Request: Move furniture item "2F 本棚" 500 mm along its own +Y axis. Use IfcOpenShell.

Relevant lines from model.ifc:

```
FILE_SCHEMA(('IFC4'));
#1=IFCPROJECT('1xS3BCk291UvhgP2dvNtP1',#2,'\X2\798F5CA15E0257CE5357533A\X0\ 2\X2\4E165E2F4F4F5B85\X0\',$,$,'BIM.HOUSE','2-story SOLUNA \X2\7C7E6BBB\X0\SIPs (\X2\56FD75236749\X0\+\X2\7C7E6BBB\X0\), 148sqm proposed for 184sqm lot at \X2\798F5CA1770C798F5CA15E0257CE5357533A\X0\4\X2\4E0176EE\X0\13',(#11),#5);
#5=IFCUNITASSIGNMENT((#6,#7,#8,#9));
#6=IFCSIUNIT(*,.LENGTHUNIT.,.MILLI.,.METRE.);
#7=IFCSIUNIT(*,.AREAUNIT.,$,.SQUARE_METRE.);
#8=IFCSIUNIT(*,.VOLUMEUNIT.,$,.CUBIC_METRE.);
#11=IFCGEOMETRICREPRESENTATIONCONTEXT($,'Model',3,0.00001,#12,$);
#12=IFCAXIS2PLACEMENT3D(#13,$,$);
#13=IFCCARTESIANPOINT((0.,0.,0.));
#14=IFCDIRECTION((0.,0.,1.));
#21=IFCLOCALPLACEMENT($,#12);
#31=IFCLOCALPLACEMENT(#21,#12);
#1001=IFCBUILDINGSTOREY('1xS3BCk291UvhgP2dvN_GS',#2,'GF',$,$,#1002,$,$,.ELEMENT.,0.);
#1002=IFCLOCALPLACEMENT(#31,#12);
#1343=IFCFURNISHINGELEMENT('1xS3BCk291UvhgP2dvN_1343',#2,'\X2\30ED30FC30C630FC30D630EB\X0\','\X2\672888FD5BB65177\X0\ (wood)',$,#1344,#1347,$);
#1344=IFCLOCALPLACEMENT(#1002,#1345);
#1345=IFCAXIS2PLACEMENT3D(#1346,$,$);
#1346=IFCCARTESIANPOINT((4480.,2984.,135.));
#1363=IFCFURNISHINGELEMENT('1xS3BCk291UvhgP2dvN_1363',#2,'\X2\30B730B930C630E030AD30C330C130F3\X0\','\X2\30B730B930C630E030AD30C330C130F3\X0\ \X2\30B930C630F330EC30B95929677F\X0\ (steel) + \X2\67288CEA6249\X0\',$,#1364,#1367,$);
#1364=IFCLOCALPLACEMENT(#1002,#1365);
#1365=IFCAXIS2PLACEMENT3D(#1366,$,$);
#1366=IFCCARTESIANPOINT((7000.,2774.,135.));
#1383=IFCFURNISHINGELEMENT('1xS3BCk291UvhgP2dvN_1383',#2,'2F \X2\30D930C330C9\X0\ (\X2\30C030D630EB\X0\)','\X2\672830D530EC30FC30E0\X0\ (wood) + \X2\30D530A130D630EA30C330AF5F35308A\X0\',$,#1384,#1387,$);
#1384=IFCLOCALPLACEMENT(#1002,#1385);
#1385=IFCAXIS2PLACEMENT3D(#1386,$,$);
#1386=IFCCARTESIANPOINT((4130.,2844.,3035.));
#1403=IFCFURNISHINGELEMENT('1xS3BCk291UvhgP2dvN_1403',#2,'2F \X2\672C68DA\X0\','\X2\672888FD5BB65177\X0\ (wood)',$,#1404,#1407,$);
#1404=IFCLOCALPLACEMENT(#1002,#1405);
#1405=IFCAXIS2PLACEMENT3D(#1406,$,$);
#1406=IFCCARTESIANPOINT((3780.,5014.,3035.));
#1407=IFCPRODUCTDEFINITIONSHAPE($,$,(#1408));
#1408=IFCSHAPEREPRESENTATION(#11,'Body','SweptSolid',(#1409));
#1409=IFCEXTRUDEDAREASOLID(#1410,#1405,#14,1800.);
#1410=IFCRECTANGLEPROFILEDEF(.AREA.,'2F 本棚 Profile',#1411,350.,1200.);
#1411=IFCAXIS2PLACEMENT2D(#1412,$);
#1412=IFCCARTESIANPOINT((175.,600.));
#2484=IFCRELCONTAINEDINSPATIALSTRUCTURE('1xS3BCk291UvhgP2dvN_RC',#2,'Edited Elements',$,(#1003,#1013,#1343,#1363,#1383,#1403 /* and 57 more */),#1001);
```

```python
import ifcopenshell
import ifcopenshell.api.geometry
import ifcopenshell.util.placement
import ifcopenshell.util.unit

model = ifcopenshell.open("model.ifc")
unit_scale = ifcopenshell.util.unit.calculate_unit_scale(model)

item = model.by_guid("1xS3BCk291UvhgP2dvN_1403")
matrix = ifcopenshell.util.placement.get_local_placement(item.ObjectPlacement)
matrix[:3, 3] += matrix[:3, 1] * 0.5 / unit_scale
ifcopenshell.api.geometry.edit_object_placement(model, product=item, matrix=matrix, is_si=False)

print(ifcopenshell.util.placement.get_local_placement(item.ObjectPlacement).round(3) + 0.0)

model.write("model_updated.ifc")
```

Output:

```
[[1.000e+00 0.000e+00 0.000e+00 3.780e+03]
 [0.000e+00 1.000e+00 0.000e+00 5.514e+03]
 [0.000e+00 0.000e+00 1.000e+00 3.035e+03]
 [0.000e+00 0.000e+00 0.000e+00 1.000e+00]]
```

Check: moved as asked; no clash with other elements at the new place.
